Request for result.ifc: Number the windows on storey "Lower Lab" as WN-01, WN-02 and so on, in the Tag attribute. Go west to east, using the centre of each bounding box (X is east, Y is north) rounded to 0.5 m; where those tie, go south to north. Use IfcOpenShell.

First a look at what the model holds.

```python
import ifcopenshell
import ifcopenshell.util.element
import ifcopenshell.util.placement

model = ifcopenshell.open("result.ifc")
print(model.schema)
storey = next(s for s in model.by_type("IfcBuildingStorey") if s.Name == "Lower Lab")
windows = [e for e in ifcopenshell.util.element.get_decomposition(storey) if e.is_a("IfcWindow")]
for e in sorted(windows, key=lambda e: e.id()):
    origin = ifcopenshell.util.placement.get_local_placement(e.ObjectPlacement)[:3, 3]
    print(e.id(), e.Tag, e.Name, origin.round(2) + 0.0, sep=" | ")
```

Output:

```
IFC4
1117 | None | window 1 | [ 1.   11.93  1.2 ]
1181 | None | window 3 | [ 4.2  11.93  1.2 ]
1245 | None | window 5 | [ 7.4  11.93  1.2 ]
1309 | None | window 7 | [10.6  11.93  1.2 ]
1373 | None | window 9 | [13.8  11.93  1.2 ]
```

```python
import ifcopenshell
import ifcopenshell.geom
import ifcopenshell.util.element
import ifcopenshell.util.shape

model = ifcopenshell.open("result.ifc")
settings = ifcopenshell.geom.settings()
settings.set("use-world-coords", True)


def centre(element):
    shape = ifcopenshell.geom.create_shape(settings, element)
    return ifcopenshell.util.shape.get_bbox_centroid(shape.geometry)


storey = next(s for s in model.by_type("IfcBuildingStorey") if s.Name == "Lower Lab")
windows = [e for e in ifcopenshell.util.element.get_decomposition(storey) if e.is_a("IfcWindow")]

# Insertion points can sit at a corner or the storey origin, so sort by the geometry (in metres).
centres = {e: centre(e) for e in windows}
windows.sort(key=lambda e: (round(centres[e][0] / 0.5), centres[e][1]))

for i, e in enumerate(windows, start=1):
    number = f"WN-{i:02d}"
    e.Tag = number
    print(e.id(), number)

model.write("result-out.ifc")
```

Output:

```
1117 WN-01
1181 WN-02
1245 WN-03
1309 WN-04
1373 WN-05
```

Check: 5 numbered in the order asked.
